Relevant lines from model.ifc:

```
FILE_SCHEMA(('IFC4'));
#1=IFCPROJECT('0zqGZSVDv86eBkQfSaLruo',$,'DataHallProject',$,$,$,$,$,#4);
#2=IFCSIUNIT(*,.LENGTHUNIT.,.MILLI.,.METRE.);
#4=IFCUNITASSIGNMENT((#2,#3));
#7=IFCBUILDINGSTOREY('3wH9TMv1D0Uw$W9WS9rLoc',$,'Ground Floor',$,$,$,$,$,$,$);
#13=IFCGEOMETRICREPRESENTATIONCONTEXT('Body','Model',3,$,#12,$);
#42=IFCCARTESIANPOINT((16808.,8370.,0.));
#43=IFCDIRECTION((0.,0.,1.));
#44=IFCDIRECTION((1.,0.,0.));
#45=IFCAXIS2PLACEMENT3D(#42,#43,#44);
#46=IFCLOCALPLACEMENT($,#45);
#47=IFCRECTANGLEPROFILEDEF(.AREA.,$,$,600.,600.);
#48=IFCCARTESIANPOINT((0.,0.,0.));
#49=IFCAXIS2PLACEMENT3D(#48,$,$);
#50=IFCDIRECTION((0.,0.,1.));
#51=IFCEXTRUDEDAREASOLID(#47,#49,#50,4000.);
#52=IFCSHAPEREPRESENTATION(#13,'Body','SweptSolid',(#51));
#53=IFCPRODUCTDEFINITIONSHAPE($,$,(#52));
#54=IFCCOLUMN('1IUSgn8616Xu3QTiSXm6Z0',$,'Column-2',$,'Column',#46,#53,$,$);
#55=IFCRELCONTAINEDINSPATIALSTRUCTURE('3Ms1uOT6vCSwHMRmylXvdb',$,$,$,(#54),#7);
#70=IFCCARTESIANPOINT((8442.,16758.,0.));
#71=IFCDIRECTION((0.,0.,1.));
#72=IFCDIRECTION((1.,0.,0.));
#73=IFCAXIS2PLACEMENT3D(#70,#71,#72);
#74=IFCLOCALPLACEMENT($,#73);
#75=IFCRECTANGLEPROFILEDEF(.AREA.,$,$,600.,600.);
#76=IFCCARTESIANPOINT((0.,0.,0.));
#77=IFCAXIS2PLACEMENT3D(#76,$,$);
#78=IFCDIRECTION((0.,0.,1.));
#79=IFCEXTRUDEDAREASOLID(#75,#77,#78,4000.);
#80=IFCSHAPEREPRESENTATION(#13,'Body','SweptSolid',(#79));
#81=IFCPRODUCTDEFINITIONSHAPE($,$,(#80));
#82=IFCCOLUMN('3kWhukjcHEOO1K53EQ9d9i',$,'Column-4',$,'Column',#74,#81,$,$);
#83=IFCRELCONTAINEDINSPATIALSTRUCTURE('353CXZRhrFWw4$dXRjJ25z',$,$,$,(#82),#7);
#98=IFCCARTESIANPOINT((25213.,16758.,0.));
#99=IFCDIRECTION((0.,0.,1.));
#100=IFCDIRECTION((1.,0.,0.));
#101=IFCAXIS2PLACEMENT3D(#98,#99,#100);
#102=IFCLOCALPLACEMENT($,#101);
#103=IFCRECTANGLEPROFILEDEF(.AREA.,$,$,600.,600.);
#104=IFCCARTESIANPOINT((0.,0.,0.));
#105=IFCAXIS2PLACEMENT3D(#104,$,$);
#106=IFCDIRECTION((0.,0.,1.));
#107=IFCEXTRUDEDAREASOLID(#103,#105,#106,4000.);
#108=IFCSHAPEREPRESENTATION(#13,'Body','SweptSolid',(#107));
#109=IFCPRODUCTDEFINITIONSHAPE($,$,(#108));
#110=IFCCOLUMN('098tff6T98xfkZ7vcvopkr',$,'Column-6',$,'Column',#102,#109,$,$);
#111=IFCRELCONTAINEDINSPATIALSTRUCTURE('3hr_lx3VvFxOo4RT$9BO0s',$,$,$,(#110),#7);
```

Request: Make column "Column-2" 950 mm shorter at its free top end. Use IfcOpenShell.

```python
import ifcopenshell

model = ifcopenshell.open("model.ifc")

member = model.by_guid("1IUSgn8616Xu3QTiSXm6Z0")
change = -950.0

# The extrusion runs towards the end named, so only its depth changes.
body = next(r for r in member.Representation.Representations if r.RepresentationIdentifier == "Body")
solid = body.Items[0]
old_length = solid.Depth
solid.Depth += change

print(f"length {old_length:g} -> {solid.Depth:g}")

model.write("model_edited.ifc")
```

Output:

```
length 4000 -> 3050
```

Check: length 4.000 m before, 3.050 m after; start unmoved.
